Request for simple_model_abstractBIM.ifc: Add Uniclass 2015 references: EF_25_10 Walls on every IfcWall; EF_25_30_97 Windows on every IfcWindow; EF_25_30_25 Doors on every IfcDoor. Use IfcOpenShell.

First a look at what the model holds.

```python
import ifcopenshell

model = ifcopenshell.open("simple_model_abstractBIM.ifc")
print(model.schema)
print("classifications:", [c.Name for c in model.by_type("IfcClassification")])
for ifc_class in ("IfcDoor", "IfcRoof", "IfcStair", "IfcWall", "IfcWindow"):
    print(ifc_class, len(model.by_type(ifc_class)))
```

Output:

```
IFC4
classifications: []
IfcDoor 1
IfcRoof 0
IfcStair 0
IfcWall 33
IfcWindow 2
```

```python
import ifcopenshell
import ifcopenshell.api.classification

model = ifcopenshell.open("simple_model_abstractBIM.ifc")

system = ifcopenshell.api.classification.add_classification(model, classification="Uniclass 2015")

codes = {
    "IfcWall": ("EF_25_10", "Walls"),
    "IfcWindow": ("EF_25_30_97", "Windows"),
    "IfcDoor": ("EF_25_30_25", "Doors"),
}
for ifc_class, (code, name) in codes.items():
    products = model.by_type(ifc_class)
    ifcopenshell.api.classification.add_reference(
        model, products=products, classification=system, identification=code, name=name
    )
    print(code, len(products))

model.write("simple_model_abstractBIM_updated.ifc")
```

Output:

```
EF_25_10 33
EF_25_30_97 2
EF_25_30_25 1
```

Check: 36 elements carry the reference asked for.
